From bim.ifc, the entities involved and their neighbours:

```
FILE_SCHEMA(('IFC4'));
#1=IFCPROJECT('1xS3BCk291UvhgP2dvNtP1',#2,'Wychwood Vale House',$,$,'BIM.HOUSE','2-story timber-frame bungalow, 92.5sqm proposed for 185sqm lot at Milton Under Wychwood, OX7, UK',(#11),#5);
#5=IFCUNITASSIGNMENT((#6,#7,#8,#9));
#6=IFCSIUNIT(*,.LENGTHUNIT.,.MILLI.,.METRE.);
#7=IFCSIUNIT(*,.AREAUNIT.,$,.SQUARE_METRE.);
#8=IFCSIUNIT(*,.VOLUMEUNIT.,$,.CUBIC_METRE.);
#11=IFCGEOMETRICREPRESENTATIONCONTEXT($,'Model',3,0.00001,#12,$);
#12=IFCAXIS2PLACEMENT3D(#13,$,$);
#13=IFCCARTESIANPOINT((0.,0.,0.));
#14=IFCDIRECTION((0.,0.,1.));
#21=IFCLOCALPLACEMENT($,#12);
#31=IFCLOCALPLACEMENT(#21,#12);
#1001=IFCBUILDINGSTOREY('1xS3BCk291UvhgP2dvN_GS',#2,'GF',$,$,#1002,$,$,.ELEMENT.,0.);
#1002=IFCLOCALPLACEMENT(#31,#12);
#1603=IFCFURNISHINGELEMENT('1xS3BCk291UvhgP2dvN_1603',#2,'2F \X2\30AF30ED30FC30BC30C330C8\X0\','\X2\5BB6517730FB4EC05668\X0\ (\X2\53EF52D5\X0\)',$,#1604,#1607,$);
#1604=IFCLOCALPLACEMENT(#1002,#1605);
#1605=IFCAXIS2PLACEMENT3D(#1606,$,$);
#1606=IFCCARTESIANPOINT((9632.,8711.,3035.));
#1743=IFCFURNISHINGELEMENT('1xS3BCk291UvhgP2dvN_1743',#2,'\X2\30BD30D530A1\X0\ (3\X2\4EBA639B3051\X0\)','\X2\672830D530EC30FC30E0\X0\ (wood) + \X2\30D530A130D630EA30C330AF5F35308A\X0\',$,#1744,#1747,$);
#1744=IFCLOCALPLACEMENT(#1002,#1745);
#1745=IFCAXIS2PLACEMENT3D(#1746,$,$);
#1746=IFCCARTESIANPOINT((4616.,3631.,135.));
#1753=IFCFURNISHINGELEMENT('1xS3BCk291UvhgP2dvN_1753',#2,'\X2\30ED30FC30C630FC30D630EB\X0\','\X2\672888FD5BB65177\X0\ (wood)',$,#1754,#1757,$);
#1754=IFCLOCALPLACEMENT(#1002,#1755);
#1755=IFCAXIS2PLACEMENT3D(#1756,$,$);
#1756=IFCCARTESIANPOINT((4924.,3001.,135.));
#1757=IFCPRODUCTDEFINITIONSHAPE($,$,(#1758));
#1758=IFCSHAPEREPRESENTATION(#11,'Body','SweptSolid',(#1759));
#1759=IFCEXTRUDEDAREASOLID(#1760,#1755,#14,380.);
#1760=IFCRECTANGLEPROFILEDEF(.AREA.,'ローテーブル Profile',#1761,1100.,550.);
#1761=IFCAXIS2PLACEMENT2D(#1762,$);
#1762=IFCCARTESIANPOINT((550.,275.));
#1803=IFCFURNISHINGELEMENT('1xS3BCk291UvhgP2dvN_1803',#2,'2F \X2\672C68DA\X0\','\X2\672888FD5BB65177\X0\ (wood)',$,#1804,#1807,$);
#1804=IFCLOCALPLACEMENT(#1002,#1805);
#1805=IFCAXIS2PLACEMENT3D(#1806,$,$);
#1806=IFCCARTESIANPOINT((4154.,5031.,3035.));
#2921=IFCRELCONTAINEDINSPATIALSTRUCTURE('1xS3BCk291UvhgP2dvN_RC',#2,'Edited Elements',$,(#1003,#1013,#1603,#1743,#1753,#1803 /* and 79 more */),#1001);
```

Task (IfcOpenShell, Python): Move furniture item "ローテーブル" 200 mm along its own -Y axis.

```python
import ifcopenshell
import ifcopenshell.api.geometry
import ifcopenshell.util.placement
import ifcopenshell.util.unit

model = ifcopenshell.open("bim.ifc")
unit_scale = ifcopenshell.util.unit.calculate_unit_scale(model)

item = model.by_guid("1xS3BCk291UvhgP2dvN_1753")
matrix = ifcopenshell.util.placement.get_local_placement(item.ObjectPlacement)
matrix[:3, 3] -= matrix[:3, 1] * 0.2 / unit_scale
ifcopenshell.api.geometry.edit_object_placement(model, product=item, matrix=matrix, is_si=False)

print(ifcopenshell.util.placement.get_local_placement(item.ObjectPlacement).round(3) + 0.0)

model.write("bim_edited.ifc")
```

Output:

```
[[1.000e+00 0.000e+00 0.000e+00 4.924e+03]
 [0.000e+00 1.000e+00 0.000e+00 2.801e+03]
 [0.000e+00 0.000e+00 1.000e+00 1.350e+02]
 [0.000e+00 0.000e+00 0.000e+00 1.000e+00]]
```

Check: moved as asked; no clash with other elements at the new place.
